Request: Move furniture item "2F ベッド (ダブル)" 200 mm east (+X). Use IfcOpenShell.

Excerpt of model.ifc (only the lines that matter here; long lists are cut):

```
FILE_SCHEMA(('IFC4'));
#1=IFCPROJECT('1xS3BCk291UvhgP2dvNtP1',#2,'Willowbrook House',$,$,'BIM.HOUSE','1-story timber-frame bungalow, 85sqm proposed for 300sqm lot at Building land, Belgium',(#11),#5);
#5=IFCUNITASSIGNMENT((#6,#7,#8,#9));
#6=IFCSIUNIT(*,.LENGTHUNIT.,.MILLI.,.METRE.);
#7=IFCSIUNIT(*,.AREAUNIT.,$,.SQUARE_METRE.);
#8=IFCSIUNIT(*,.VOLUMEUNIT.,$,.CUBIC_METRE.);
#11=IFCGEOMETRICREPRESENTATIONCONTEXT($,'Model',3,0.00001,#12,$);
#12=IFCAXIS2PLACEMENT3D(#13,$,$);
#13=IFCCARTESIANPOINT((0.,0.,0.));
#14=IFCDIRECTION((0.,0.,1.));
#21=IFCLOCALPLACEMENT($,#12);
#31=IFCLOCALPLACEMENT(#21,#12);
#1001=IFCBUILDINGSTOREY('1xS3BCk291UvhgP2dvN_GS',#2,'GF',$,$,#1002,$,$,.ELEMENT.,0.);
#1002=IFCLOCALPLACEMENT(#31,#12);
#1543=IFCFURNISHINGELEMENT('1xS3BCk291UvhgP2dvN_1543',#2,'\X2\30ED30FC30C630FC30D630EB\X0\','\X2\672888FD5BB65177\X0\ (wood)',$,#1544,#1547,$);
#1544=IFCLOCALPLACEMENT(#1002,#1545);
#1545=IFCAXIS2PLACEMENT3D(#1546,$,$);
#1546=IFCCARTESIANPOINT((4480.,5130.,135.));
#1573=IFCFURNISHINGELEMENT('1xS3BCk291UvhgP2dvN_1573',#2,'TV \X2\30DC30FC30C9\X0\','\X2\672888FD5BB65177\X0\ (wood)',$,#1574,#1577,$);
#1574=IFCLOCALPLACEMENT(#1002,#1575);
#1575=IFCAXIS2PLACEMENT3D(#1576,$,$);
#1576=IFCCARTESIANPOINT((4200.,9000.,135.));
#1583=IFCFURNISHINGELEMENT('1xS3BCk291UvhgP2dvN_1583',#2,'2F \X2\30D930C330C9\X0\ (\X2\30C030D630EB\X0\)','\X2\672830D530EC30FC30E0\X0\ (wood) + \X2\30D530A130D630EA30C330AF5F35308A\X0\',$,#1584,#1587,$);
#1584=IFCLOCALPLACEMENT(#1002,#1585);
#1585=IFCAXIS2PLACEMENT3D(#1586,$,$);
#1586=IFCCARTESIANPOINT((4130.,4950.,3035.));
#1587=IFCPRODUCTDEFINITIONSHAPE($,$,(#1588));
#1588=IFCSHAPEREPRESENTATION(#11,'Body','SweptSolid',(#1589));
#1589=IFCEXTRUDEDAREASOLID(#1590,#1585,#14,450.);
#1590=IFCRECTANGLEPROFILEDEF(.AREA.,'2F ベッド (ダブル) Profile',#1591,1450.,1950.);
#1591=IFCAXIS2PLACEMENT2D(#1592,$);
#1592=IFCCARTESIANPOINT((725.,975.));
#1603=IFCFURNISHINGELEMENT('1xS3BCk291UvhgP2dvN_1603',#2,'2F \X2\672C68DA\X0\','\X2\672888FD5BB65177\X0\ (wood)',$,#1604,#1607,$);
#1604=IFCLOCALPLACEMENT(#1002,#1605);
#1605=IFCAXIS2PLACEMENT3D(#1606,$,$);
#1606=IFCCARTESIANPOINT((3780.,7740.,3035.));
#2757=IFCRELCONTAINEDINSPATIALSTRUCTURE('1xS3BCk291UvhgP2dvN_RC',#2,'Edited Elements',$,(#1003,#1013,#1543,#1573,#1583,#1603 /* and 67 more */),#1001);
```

```python
import ifcopenshell
import ifcopenshell.api.geometry
import ifcopenshell.util.placement
import ifcopenshell.util.unit

model = ifcopenshell.open("model.ifc")
unit_scale = ifcopenshell.util.unit.calculate_unit_scale(model)

item = model.by_id(1583)
matrix = ifcopenshell.util.placement.get_local_placement(item.ObjectPlacement)
matrix[0, 3] += 0.2 / unit_scale
ifcopenshell.api.geometry.edit_object_placement(model, product=item, matrix=matrix, is_si=False)

print(ifcopenshell.util.placement.get_local_placement(item.ObjectPlacement).round(3) + 0.0)

model.write("model-out.ifc")
```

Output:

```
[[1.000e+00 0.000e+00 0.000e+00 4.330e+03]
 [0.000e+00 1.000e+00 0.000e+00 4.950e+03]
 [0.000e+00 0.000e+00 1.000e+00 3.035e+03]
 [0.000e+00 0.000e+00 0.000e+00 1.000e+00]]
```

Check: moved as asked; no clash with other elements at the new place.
